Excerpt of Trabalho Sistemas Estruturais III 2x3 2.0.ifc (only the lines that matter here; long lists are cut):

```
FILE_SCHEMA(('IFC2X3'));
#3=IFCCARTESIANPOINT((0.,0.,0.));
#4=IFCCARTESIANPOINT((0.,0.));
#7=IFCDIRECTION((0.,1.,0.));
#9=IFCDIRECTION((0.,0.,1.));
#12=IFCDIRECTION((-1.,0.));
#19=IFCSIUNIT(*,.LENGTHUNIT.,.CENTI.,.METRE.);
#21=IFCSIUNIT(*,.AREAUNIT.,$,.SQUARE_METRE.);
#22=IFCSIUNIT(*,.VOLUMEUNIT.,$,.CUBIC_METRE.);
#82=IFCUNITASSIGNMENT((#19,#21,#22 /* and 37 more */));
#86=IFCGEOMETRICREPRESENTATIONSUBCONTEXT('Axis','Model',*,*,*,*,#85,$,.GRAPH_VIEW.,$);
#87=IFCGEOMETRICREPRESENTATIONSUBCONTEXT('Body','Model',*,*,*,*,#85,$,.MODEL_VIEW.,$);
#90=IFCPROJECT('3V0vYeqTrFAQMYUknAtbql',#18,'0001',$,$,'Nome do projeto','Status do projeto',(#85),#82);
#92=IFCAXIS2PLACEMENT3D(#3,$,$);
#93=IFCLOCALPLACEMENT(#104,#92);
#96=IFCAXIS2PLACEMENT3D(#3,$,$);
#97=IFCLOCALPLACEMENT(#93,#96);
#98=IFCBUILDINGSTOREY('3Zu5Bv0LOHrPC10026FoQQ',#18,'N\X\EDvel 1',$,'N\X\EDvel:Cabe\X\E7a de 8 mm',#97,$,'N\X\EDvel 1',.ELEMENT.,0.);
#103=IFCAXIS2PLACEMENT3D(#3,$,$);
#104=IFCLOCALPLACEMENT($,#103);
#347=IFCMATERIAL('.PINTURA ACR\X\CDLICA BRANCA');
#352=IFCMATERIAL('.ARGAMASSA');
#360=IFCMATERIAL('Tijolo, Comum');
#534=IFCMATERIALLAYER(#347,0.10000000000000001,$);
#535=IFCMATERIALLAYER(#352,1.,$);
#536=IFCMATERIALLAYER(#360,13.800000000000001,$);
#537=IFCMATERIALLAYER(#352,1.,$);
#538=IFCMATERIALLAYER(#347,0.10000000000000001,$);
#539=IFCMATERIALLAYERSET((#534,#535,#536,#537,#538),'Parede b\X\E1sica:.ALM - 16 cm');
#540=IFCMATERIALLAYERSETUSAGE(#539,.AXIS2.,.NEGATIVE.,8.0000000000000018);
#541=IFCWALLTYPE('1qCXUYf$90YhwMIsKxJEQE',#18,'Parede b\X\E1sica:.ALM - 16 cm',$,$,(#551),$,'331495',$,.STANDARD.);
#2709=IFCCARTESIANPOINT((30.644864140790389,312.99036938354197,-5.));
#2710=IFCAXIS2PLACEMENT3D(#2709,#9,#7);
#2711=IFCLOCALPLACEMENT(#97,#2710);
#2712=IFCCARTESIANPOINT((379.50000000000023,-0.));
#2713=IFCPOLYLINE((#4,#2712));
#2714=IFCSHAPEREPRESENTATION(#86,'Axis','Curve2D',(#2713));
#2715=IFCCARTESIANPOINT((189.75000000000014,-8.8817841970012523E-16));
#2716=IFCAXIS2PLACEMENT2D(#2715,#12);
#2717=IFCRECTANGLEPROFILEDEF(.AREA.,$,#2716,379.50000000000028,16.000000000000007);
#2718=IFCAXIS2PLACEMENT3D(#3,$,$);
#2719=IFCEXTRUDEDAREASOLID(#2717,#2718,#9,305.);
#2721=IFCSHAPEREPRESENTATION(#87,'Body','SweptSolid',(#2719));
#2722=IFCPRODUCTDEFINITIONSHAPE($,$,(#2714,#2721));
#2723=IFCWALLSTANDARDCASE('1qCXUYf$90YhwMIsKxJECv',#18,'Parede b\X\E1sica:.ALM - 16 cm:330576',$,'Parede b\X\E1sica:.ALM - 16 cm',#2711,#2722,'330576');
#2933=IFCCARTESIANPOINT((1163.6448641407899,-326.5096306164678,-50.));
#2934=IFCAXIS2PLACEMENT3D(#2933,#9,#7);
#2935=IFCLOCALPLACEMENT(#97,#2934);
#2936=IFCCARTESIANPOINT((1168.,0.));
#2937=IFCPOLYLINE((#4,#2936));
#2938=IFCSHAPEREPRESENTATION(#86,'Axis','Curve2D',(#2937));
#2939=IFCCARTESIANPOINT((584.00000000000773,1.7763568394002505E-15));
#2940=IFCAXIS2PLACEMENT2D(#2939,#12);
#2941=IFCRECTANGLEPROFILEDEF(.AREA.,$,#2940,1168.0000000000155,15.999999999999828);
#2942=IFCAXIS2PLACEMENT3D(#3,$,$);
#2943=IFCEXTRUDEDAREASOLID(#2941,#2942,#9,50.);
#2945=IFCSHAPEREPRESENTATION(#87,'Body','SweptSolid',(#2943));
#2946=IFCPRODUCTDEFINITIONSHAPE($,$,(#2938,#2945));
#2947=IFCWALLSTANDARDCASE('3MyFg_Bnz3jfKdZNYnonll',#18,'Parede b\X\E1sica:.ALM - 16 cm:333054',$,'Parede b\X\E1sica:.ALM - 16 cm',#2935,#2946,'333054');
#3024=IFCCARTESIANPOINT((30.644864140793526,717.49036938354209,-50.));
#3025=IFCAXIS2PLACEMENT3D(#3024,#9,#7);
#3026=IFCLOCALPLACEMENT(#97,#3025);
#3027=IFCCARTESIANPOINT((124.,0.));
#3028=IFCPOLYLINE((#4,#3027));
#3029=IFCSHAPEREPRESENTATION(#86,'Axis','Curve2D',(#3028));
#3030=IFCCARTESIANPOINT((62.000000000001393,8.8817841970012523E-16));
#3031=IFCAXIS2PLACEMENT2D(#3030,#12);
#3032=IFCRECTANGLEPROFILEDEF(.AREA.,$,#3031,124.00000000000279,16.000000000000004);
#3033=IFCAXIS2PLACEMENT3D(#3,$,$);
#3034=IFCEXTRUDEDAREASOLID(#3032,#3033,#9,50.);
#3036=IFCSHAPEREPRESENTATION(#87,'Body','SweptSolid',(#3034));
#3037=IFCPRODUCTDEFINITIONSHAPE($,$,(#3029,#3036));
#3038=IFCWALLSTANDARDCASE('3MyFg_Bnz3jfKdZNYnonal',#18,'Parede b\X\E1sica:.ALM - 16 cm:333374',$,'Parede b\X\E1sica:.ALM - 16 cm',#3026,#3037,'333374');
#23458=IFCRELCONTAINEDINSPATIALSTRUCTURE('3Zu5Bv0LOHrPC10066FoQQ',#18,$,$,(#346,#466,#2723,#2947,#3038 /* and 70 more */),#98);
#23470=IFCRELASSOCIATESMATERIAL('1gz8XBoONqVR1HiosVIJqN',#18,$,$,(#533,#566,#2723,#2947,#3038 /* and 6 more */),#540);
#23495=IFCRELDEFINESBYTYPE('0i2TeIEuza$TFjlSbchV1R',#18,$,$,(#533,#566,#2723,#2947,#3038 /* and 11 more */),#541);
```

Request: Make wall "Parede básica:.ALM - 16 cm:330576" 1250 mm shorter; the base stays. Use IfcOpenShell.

```python
import ifcopenshell
import ifcopenshell.geom
import ifcopenshell.util.representation
import ifcopenshell.util.shape
import ifcopenshell.util.unit

model = ifcopenshell.open("Trabalho Sistemas Estruturais III 2x3 2.0.ifc")
unit_scale = ifcopenshell.util.unit.calculate_unit_scale(model)
settings = ifcopenshell.geom.settings()


def volume(element):
    """Net volume in cubic metres, openings subtracted."""
    shape = ifcopenshell.geom.create_shape(settings, element)
    return ifcopenshell.util.shape.get_volume(shape.geometry)


wall = model.by_guid("1qCXUYf$90YhwMIsKxJECv")
before = volume(wall)

body = ifcopenshell.util.representation.get_representation(wall, "Model", "Body")
solid = body.Items[0]
old_height = solid.Depth
solid.Depth -= 1.25 / unit_scale
after = volume(wall)

print(f"height {old_height:g} -> {solid.Depth:g}, volume {before:.3f} -> {after:.3f} m3")

model.write("Trabalho Sistemas Estruturais III 2x3 2.0_rev.ifc")
```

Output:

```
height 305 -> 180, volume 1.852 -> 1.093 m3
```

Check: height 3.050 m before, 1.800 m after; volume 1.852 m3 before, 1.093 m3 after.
